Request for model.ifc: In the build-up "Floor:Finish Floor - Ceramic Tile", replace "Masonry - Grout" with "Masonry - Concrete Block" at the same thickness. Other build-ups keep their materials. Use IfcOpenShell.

First a look at what the model holds.

```python
import ifcopenshell
import ifcopenshell.util.element

model = ifcopenshell.open("model.ifc")
print(model.schema)
for layer_set in model.by_type("IfcMaterialLayerSet"):
    if layer_set.LayerSetName == "Floor:Finish Floor - Ceramic Tile":
        for layer in layer_set.MaterialLayers:
            print(layer.id(), layer.Material and layer.Material.Name, layer.LayerThickness, sep=" | ")
        print(len(ifcopenshell.util.element.get_elements_by_material(model, layer_set)), "elements and types use it")
print(sorted(m.Name for m in model.by_type("IfcMaterial") if m.Name)[:60])
```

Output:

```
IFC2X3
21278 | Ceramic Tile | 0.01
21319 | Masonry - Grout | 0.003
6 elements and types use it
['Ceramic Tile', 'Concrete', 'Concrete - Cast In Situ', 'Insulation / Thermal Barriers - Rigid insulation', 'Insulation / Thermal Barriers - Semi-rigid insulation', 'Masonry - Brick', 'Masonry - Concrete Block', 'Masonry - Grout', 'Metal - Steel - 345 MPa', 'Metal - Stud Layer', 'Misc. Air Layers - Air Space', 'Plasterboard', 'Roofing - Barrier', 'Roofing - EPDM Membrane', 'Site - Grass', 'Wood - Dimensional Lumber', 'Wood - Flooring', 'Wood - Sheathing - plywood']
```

```python
import ifcopenshell
import ifcopenshell.api.material

model = ifcopenshell.open("model.ifc")

layer_set = next(s for s in model.by_type("IfcMaterialLayerSet") if s.LayerSetName == "Floor:Finish Floor - Ceramic Tile")
layer = next(l for l in layer_set.MaterialLayers if l.Material and l.Material.Name == "Masonry - Grout")
material = next(m for m in model.by_type("IfcMaterial") if m.Name == "Masonry - Concrete Block")

# Point this one layer at the other material; renaming the old one would change it everywhere.
ifcopenshell.api.material.edit_layer(model, layer=layer, attributes={}, material=material)

print([l.Material.Name if l.Material else None for l in layer_set.MaterialLayers])

model.write("model_rev.ifc")
```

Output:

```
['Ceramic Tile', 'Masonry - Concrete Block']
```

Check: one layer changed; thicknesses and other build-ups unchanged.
